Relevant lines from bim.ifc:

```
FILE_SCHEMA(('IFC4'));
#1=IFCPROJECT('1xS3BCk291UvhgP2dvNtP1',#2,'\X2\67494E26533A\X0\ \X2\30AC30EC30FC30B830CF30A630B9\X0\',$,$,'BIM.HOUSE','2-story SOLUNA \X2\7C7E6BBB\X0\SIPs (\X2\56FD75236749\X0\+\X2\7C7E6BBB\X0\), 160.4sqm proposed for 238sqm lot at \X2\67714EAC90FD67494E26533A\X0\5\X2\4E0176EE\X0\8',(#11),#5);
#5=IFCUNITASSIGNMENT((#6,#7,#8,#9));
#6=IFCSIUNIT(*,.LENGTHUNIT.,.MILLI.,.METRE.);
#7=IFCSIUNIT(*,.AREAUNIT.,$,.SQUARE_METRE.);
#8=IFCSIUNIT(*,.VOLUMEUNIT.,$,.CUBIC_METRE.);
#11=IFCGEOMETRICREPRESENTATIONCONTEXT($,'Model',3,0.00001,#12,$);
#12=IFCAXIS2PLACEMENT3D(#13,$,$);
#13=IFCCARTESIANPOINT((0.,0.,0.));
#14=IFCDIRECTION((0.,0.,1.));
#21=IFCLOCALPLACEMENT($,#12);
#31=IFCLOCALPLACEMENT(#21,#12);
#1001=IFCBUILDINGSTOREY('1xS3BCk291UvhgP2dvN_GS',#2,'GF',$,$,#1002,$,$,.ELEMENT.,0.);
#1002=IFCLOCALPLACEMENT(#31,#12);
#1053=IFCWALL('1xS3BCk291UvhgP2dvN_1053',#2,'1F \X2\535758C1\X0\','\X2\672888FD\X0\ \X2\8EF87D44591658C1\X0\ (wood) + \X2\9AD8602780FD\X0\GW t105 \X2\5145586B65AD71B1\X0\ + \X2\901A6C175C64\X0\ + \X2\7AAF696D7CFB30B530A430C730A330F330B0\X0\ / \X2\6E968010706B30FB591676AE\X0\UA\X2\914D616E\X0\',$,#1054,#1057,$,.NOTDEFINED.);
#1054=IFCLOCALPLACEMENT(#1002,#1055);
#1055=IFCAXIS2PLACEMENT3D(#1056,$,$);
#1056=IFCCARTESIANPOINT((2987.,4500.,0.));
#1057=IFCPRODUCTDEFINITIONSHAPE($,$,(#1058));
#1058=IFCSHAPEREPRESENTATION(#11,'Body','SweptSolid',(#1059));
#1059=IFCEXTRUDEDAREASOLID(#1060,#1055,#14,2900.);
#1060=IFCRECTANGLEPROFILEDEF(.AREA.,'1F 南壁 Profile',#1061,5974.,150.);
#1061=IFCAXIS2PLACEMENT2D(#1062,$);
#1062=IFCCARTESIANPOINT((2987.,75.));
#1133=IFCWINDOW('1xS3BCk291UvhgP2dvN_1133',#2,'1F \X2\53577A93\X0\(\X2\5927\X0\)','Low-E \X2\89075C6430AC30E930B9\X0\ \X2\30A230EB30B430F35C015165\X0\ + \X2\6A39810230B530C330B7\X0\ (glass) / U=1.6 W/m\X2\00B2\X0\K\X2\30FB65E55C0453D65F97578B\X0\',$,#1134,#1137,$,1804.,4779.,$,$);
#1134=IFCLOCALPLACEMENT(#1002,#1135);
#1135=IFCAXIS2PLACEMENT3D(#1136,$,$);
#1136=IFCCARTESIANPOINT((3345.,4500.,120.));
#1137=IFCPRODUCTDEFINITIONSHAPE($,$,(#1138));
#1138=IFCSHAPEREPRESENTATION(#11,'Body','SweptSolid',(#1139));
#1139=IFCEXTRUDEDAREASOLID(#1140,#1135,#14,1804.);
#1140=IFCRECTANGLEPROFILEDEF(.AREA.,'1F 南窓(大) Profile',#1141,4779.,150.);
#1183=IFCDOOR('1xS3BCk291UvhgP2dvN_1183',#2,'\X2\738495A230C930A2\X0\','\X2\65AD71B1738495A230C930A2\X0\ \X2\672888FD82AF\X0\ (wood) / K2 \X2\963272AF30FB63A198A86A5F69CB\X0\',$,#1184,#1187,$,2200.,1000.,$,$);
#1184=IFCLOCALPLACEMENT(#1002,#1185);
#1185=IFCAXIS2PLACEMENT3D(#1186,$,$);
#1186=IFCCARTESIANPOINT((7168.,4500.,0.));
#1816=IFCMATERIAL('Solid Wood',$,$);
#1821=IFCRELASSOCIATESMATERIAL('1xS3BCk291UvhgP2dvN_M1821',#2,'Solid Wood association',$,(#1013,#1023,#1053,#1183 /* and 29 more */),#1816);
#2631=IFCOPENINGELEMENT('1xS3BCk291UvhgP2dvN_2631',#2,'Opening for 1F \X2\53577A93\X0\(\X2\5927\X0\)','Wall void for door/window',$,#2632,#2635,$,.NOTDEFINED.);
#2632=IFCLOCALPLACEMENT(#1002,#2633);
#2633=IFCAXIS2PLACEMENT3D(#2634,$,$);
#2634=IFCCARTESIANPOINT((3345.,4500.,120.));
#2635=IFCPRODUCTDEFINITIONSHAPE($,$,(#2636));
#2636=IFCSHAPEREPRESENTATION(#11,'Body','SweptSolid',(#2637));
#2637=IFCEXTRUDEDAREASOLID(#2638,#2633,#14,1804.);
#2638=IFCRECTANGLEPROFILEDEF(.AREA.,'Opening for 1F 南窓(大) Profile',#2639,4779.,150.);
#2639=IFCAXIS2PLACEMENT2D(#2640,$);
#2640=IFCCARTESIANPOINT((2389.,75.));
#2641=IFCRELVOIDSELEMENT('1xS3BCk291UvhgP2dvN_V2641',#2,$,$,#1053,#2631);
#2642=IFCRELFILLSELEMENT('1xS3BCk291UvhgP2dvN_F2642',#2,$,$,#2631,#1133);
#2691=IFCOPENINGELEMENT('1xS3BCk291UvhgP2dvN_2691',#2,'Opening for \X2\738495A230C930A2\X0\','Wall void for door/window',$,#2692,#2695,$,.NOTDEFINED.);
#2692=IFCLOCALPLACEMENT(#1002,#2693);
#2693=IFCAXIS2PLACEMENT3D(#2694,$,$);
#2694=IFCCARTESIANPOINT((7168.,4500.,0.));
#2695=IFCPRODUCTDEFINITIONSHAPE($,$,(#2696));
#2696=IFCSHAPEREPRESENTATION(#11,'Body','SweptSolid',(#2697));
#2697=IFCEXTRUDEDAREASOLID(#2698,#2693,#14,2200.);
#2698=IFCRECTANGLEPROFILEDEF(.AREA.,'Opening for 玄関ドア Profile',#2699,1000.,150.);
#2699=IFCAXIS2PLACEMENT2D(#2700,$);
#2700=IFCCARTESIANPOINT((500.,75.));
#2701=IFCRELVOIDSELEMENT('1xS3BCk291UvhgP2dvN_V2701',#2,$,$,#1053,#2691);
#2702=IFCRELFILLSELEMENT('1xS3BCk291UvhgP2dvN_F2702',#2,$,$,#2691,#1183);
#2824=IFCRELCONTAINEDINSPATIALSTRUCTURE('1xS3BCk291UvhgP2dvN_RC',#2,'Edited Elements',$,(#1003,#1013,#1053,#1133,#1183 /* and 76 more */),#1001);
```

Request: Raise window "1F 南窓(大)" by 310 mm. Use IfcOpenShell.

```python
import numpy as np
import ifcopenshell
import ifcopenshell.api.geometry
import ifcopenshell.util.placement
import ifcopenshell.util.unit

model = ifcopenshell.open("bim.ifc")
unit_scale = ifcopenshell.util.unit.calculate_unit_scale(model)

window = model.by_id(1133)
opening = window.FillsVoids[0].RelatingOpeningElement
dz = 0.31 / unit_scale

shift = np.array([0.0, 0.0, dz])
# The window is not placed relative to its opening, so move both.
for product in (opening, window):
    matrix = ifcopenshell.util.placement.get_local_placement(product.ObjectPlacement)
    matrix[:3, 3] += shift
    ifcopenshell.api.geometry.edit_object_placement(model, product=product, matrix=matrix, is_si=False)

print(f"moved by {dz * unit_scale:+.3f} m")

model.write("bim_rev.ifc")
```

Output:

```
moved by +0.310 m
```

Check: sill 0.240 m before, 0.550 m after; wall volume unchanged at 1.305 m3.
